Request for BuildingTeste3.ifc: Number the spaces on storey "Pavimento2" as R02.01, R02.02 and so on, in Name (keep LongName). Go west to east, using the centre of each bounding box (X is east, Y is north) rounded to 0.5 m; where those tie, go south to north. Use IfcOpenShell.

First a look at what the model holds.

```python
import ifcopenshell
import ifcopenshell.util.element
import ifcopenshell.util.placement

model = ifcopenshell.open("BuildingTeste3.ifc")
print(model.schema)
storey = next(s for s in model.by_type("IfcBuildingStorey") if s.Name == "Pavimento2")
spaces = [e for e in ifcopenshell.util.element.get_decomposition(storey) if e.is_a("IfcSpace")]
for e in sorted(spaces, key=lambda e: e.id()):
    origin = ifcopenshell.util.placement.get_local_placement(e.ObjectPlacement)[:3, 3]
    print(e.id(), e.Name, e.LongName, origin.round(2) + 0.0, sep=" | ")
```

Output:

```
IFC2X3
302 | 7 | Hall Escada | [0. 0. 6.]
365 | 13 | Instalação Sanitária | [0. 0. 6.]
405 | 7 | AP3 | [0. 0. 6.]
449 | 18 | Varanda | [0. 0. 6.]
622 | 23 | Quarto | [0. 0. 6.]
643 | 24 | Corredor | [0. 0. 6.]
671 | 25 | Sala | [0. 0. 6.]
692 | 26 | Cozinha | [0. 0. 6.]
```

```python
import ifcopenshell
import ifcopenshell.geom
import ifcopenshell.util.element
import ifcopenshell.util.shape

model = ifcopenshell.open("BuildingTeste3.ifc")
settings = ifcopenshell.geom.settings()
settings.set("use-world-coords", True)


def centre(element):
    shape = ifcopenshell.geom.create_shape(settings, element)
    return ifcopenshell.util.shape.get_bbox_centroid(shape.geometry)


storey = next(s for s in model.by_type("IfcBuildingStorey") if s.Name == "Pavimento2")
spaces = [e for e in ifcopenshell.util.element.get_decomposition(storey) if e.is_a("IfcSpace")]

# Insertion points can sit at a corner or the storey origin, so sort by the geometry (in metres).
centres = {e: centre(e) for e in spaces}
spaces.sort(key=lambda e: (round(centres[e][0] / 0.5), centres[e][1]))

for i, e in enumerate(spaces, start=1):
    number = f"R02.{i:02d}"
    e.Name = number
    print(e.id(), number)

model.write("BuildingTeste3_updated.ifc")
```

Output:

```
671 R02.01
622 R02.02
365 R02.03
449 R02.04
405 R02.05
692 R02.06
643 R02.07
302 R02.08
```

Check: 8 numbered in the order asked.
